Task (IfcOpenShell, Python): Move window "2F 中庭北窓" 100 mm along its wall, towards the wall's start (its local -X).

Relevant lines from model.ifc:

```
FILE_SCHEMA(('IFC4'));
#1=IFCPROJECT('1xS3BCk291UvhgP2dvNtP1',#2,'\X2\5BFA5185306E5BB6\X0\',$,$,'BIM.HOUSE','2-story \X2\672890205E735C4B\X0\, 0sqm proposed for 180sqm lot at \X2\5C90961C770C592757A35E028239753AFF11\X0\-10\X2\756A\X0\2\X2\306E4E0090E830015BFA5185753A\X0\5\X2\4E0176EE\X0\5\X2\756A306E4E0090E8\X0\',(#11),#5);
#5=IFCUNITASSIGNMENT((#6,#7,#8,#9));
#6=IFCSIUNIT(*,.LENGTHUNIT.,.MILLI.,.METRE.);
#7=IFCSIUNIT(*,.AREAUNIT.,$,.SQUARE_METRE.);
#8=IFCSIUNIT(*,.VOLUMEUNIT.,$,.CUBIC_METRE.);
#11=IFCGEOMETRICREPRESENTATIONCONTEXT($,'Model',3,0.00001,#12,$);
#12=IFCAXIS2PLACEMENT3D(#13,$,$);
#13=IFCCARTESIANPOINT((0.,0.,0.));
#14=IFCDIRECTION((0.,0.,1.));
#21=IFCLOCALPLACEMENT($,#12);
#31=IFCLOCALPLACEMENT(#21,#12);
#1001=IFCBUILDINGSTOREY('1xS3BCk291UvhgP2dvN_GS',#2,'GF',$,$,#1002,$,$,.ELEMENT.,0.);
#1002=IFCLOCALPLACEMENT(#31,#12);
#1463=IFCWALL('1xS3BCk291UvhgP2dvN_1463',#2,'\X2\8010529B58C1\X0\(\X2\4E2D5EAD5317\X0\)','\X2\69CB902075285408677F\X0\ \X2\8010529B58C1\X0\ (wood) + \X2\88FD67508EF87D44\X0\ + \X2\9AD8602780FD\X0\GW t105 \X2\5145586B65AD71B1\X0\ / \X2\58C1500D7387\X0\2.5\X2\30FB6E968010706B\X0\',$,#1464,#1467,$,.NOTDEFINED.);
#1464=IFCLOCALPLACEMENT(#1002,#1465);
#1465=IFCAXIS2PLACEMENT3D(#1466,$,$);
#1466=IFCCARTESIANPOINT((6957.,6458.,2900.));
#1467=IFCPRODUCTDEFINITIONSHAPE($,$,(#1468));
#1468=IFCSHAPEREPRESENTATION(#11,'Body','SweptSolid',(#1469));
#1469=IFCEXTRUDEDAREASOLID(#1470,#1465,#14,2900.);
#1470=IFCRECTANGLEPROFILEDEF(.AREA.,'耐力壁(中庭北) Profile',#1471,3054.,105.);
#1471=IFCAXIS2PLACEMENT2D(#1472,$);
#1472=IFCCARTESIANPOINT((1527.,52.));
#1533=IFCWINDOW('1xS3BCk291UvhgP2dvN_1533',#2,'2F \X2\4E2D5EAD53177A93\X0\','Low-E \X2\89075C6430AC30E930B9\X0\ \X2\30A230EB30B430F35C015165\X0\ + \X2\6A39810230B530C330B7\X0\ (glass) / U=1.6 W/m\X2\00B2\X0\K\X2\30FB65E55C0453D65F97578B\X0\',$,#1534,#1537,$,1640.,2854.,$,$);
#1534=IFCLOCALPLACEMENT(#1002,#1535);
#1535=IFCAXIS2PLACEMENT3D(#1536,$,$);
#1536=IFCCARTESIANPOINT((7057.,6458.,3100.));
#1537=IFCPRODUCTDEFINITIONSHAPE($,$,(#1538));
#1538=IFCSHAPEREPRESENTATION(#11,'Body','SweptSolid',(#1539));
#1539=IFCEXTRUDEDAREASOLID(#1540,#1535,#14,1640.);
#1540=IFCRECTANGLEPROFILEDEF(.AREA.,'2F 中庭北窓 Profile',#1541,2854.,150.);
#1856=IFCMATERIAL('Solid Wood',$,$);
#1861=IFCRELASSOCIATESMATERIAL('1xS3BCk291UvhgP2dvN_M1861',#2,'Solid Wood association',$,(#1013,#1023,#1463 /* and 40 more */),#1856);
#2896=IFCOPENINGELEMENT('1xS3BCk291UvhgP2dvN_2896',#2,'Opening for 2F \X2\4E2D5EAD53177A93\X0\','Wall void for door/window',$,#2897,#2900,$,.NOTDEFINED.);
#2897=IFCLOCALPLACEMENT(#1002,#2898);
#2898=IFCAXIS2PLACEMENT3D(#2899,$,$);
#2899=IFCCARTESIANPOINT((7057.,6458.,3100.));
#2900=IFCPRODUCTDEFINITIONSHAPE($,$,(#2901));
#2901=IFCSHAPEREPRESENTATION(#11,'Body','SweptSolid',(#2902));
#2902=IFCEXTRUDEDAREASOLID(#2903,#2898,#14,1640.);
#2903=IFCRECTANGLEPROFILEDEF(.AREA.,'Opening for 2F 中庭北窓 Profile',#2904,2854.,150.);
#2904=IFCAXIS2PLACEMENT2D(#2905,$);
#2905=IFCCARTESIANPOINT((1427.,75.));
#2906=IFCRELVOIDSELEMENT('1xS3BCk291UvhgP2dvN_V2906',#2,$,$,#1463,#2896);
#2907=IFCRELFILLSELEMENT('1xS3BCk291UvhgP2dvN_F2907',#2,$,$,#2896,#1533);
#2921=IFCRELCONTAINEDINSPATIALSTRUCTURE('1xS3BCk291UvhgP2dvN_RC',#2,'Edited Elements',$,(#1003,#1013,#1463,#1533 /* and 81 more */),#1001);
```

```python
import ifcopenshell
import ifcopenshell.api.geometry
import ifcopenshell.util.placement
import ifcopenshell.util.unit

model = ifcopenshell.open("model.ifc")
unit_scale = ifcopenshell.util.unit.calculate_unit_scale(model)

window = model.by_guid("1xS3BCk291UvhgP2dvN_1533")
opening = window.FillsVoids[0].RelatingOpeningElement
wall = opening.VoidsElements[0].RelatingBuildingElement

wall_matrix = ifcopenshell.util.placement.get_local_placement(wall.ObjectPlacement)
shift = wall_matrix[:3, 0] * -0.1 / unit_scale
before = ifcopenshell.util.placement.get_local_placement(window.ObjectPlacement)[:3, 3].copy()

# The window is not placed relative to its opening, so move both.
for product in (opening, window):
    matrix = ifcopenshell.util.placement.get_local_placement(product.ObjectPlacement)
    matrix[:3, 3] += shift
    ifcopenshell.api.geometry.edit_object_placement(model, product=product, matrix=matrix, is_si=False)

after = ifcopenshell.util.placement.get_local_placement(window.ObjectPlacement)[:3, 3]
print("window moved by", (after - before).round(3) + 0.0)

model.write("model_edited.ifc")
```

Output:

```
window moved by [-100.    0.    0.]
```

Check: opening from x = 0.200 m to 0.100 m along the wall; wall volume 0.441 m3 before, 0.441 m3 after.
